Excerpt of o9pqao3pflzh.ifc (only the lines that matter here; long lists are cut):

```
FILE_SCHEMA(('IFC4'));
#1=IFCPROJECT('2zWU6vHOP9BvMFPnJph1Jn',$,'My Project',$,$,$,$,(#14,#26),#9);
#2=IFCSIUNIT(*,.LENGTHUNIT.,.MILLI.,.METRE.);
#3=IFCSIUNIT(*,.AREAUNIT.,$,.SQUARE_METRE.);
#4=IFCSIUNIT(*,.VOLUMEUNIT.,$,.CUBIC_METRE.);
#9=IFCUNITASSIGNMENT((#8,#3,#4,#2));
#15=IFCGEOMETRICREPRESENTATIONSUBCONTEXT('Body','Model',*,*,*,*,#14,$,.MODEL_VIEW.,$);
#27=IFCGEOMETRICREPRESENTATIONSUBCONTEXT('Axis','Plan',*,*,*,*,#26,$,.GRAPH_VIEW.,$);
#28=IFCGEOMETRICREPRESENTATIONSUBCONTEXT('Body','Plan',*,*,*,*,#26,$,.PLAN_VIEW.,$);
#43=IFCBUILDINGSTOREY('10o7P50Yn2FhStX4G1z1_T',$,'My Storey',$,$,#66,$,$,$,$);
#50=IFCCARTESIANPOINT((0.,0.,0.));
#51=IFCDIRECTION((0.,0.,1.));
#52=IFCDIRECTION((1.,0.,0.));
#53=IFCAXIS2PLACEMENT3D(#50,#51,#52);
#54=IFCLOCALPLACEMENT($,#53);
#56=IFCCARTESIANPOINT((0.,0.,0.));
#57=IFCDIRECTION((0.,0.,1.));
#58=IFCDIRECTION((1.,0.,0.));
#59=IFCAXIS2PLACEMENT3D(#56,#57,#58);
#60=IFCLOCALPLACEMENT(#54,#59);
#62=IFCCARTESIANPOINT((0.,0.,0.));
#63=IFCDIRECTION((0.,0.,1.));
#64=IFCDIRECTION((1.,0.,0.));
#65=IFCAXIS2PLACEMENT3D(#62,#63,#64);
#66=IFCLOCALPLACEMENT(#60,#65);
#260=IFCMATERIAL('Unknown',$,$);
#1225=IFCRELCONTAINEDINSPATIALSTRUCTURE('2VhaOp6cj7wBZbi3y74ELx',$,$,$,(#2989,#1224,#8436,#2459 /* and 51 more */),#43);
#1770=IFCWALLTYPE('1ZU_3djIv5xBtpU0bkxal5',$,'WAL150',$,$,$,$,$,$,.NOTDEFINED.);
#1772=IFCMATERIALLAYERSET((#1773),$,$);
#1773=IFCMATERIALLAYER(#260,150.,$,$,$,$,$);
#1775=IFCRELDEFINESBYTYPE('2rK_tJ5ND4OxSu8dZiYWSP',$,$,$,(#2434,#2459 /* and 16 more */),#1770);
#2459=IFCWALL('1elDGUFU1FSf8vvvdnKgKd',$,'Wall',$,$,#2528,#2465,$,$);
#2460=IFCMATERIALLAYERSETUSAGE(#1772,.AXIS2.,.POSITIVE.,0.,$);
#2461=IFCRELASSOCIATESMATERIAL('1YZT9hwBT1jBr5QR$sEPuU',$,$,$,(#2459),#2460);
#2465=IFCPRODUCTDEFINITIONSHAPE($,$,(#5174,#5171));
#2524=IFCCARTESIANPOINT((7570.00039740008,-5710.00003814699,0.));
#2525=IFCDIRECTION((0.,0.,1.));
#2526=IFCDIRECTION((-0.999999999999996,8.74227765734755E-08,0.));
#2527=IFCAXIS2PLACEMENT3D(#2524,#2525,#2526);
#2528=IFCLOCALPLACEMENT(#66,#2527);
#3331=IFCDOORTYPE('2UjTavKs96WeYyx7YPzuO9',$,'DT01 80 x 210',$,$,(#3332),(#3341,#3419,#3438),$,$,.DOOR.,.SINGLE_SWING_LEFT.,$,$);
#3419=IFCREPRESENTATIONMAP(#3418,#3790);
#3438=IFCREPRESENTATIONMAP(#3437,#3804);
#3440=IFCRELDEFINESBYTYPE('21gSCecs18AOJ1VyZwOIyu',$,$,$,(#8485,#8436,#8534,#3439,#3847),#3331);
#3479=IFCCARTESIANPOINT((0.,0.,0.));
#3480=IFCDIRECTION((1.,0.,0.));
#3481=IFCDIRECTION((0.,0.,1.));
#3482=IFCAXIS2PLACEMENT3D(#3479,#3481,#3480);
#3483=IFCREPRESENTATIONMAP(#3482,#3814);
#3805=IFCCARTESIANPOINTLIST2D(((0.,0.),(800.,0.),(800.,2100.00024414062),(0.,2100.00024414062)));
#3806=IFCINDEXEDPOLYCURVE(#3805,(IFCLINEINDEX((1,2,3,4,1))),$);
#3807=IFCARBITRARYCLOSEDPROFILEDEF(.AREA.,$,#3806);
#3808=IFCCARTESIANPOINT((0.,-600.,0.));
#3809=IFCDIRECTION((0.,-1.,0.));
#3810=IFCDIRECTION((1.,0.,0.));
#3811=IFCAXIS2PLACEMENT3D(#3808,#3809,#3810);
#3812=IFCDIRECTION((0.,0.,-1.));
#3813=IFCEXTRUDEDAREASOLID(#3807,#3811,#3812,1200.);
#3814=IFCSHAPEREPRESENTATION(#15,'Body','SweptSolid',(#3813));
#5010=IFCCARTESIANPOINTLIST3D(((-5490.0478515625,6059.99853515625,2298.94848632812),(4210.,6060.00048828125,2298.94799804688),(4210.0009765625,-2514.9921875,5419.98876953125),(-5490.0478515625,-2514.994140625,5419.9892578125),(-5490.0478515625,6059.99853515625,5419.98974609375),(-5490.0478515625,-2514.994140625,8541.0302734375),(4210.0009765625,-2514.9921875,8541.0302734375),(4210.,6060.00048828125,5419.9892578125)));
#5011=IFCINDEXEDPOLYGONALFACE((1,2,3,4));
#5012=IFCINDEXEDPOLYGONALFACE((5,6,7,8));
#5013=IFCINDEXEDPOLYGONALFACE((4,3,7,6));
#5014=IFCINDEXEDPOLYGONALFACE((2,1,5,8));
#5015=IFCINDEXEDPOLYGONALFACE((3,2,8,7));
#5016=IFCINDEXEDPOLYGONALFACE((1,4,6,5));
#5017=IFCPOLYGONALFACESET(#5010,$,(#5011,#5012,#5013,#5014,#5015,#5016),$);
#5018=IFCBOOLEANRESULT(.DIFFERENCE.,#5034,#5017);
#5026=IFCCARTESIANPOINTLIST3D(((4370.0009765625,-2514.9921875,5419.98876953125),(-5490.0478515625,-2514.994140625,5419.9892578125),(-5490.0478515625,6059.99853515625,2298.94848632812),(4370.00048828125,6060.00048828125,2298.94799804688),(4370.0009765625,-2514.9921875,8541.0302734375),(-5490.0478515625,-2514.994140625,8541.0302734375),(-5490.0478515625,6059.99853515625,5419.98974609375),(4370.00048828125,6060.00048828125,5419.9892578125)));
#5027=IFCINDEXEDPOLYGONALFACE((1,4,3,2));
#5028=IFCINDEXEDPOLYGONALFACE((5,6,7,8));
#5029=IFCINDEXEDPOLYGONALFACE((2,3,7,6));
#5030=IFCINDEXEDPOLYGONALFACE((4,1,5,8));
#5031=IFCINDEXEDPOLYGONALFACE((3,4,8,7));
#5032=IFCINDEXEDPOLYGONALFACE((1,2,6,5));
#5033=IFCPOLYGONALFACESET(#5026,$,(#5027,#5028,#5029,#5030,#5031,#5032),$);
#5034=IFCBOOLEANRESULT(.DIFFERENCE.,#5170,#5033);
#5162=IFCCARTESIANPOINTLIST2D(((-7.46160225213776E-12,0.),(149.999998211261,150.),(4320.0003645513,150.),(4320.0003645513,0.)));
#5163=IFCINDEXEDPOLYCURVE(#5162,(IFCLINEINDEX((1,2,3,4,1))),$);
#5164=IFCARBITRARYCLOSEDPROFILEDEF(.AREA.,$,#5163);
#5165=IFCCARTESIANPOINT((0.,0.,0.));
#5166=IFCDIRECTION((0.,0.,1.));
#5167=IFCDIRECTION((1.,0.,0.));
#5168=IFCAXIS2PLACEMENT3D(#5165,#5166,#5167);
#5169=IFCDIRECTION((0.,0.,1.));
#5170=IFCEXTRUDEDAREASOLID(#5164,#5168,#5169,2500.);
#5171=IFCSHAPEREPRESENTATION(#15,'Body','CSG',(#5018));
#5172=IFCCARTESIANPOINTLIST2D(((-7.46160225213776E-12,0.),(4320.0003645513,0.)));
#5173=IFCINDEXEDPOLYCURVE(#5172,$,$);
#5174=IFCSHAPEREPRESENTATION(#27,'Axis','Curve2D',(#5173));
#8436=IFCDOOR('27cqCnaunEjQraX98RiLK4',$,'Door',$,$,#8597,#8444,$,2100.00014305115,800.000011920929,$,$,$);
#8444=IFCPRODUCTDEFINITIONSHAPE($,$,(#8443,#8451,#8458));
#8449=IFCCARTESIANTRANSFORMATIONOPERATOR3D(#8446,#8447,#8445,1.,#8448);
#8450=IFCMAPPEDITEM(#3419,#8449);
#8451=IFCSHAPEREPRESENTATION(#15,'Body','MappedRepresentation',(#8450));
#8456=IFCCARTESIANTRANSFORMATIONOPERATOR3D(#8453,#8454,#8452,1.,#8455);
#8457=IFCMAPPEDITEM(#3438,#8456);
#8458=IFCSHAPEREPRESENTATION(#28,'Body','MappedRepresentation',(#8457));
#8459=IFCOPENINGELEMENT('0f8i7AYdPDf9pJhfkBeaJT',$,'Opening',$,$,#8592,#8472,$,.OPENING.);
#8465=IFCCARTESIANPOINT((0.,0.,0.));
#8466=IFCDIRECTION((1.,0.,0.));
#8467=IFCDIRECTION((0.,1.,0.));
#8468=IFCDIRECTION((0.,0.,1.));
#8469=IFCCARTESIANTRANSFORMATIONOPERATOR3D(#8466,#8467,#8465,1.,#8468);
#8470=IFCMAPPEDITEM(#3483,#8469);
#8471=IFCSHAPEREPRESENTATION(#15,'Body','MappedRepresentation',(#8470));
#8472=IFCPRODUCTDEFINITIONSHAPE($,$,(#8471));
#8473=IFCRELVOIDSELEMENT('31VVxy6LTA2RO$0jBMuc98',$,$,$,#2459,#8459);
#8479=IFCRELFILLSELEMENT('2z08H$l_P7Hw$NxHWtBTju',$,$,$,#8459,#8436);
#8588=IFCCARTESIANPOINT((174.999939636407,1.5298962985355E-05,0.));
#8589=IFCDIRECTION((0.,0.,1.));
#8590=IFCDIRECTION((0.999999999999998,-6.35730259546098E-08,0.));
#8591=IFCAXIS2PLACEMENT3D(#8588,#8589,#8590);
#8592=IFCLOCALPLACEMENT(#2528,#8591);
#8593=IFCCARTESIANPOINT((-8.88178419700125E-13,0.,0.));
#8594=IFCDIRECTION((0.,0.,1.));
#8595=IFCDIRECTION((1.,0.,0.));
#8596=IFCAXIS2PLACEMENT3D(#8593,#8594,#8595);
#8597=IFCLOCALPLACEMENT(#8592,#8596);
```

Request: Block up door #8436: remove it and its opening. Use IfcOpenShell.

```python
import ifcopenshell
import ifcopenshell.api.feature
import ifcopenshell.api.root
import ifcopenshell.geom
import ifcopenshell.util.shape

model = ifcopenshell.open("o9pqao3pflzh.ifc")
settings = ifcopenshell.geom.settings()


def volume(element):
    """Net volume in cubic metres, openings subtracted."""
    shape = ifcopenshell.geom.create_shape(settings, element)
    return ifcopenshell.util.shape.get_volume(shape.geometry)


door = model.by_id(8436)
opening = door.FillsVoids[0].RelatingOpeningElement
wall = opening.VoidsElements[0].RelatingBuildingElement
before = volume(wall)

ifcopenshell.api.root.remove_product(model, product=door)
ifcopenshell.api.feature.remove_feature(model, feature=opening)

after = volume(wall)

print(f"wall volume {before:.3f} -> {after:.3f} m3")

model.write("o9pqao3pflzh_v2.ifc")
```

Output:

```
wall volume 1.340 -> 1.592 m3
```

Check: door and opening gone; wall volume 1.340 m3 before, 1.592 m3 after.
